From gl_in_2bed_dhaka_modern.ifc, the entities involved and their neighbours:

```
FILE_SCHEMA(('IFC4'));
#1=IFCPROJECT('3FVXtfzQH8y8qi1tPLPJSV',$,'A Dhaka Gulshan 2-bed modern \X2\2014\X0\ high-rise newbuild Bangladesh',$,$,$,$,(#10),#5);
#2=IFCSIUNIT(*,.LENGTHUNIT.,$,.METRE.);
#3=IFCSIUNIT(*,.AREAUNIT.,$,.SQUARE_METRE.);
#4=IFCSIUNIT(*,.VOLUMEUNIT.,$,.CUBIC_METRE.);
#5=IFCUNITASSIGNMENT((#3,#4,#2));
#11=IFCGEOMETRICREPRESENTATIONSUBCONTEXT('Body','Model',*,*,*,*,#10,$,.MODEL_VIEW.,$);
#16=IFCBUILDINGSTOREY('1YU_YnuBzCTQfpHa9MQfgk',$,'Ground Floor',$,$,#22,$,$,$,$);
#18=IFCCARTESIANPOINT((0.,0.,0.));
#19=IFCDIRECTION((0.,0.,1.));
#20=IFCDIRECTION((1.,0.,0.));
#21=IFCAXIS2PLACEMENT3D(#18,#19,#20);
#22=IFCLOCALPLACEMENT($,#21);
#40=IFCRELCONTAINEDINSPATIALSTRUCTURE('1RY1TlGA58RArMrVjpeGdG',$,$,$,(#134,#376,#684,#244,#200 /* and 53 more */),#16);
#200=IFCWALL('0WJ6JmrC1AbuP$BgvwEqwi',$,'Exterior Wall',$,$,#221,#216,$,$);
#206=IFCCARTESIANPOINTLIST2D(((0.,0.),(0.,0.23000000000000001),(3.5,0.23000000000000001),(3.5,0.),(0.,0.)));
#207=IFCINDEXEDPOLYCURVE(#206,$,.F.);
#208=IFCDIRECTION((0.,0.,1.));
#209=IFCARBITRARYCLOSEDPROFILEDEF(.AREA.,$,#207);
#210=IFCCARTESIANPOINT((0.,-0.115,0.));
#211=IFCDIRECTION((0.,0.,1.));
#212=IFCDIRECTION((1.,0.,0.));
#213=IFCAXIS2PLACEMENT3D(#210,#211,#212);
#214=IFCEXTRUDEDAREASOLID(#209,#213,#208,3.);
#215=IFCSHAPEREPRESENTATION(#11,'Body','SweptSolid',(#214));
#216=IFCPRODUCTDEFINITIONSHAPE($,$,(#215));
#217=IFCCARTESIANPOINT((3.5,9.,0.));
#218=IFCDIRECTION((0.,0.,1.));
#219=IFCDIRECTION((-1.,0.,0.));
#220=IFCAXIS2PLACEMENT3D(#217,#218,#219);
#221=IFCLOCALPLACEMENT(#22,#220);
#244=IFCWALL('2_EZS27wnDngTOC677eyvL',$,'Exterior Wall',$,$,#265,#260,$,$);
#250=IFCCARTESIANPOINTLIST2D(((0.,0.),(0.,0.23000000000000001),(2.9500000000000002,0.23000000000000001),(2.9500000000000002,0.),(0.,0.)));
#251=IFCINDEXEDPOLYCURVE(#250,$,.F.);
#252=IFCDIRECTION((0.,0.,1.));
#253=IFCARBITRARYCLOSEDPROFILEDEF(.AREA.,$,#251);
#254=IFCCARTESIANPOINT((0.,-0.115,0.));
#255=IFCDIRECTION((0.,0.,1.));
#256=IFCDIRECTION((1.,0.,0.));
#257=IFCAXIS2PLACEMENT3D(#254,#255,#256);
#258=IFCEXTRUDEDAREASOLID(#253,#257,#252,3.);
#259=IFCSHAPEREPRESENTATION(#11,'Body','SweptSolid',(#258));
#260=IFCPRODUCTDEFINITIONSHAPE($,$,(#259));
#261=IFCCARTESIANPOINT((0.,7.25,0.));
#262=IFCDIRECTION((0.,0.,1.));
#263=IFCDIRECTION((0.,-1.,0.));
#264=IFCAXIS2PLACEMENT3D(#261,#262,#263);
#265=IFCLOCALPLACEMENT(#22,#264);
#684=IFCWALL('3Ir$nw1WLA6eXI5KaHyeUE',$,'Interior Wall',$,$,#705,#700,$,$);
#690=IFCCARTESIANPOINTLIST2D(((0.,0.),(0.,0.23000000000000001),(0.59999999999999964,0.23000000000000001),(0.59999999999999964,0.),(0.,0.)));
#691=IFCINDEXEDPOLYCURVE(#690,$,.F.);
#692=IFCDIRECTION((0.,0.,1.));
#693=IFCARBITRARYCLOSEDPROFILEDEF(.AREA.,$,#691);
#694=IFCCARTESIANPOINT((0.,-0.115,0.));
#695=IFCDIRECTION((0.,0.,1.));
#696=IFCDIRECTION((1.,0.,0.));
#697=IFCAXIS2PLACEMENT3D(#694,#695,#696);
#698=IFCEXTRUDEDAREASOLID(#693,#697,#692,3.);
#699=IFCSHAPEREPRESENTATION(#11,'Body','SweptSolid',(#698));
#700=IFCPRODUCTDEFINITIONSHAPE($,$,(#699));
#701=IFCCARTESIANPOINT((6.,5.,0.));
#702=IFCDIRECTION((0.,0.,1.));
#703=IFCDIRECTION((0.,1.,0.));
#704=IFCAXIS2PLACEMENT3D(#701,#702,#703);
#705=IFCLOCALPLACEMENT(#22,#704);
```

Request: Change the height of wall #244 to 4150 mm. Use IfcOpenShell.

```python
import ifcopenshell
import ifcopenshell.geom
import ifcopenshell.util.representation
import ifcopenshell.util.shape

model = ifcopenshell.open("gl_in_2bed_dhaka_modern.ifc")
settings = ifcopenshell.geom.settings()


def volume(element):
    """Net volume in cubic metres, openings subtracted."""
    shape = ifcopenshell.geom.create_shape(settings, element)
    return ifcopenshell.util.shape.get_volume(shape.geometry)


wall = model.by_guid("2_EZS27wnDngTOC677eyvL")
before = volume(wall)

body = ifcopenshell.util.representation.get_representation(wall, "Model", "Body")
solid = body.Items[0]
old_height = solid.Depth
solid.Depth = 4.15
after = volume(wall)

print(f"height {old_height:g} -> {solid.Depth:g}, volume {before:.3f} -> {after:.3f} m3")

model.write("gl_in_2bed_dhaka_modern_edited.ifc")
```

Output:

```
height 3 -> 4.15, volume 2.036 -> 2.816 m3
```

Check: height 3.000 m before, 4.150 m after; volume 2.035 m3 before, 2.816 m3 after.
